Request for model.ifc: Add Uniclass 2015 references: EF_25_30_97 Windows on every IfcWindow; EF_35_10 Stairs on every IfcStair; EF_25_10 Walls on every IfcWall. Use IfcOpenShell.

First a look at what the model holds.

```python
import ifcopenshell

model = ifcopenshell.open("model.ifc")
print(model.schema)
print("classifications:", [c.Name for c in model.by_type("IfcClassification")])
for ifc_class in ("IfcDoor", "IfcRoof", "IfcStair", "IfcWall", "IfcWindow"):
    print(ifc_class, len(model.by_type(ifc_class)))
```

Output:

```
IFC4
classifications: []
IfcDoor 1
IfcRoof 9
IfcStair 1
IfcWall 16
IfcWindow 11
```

```python
import ifcopenshell
import ifcopenshell.api.classification

model = ifcopenshell.open("model.ifc")

system = ifcopenshell.api.classification.add_classification(model, classification="Uniclass 2015")

codes = {
    "IfcWindow": ("EF_25_30_97", "Windows"),
    "IfcStair": ("EF_35_10", "Stairs"),
    "IfcWall": ("EF_25_10", "Walls"),
}
for ifc_class, (code, name) in codes.items():
    products = model.by_type(ifc_class)
    ifcopenshell.api.classification.add_reference(
        model, products=products, classification=system, identification=code, name=name
    )
    print(code, len(products))

model.write("model_edited.ifc")
```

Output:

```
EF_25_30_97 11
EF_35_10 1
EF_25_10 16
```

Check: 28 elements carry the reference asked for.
